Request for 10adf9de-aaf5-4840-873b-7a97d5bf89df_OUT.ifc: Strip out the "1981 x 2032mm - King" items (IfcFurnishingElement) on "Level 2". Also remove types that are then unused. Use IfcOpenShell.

First a look at what the model holds.

```python
import ifcopenshell
import ifcopenshell.util.element

model = ifcopenshell.open("10adf9de-aaf5-4840-873b-7a97d5bf89df_OUT.ifc")
print(model.schema)
storey = next(s for s in model.by_type("IfcBuildingStorey") if s.Name == "Level 2")
furniture = [e for e in ifcopenshell.util.element.get_decomposition(storey) if e.is_a("IfcFurnishingElement")]
seen = {}
for e in furniture:
    element_type = ifcopenshell.util.element.get_type(e)
    name = element_type.Name if element_type not in (None, e) else None
    seen[name] = seen.get(name, 0) + 1
for name, count in sorted(seen.items(), key=str):
    print(count, "x", name)
```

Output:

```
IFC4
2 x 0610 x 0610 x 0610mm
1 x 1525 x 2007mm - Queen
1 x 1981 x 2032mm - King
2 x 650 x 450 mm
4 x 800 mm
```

```python
import ifcopenshell
import ifcopenshell.api.root
import ifcopenshell.util.element

model = ifcopenshell.open("10adf9de-aaf5-4840-873b-7a97d5bf89df_OUT.ifc")

storey = next(s for s in model.by_type("IfcBuildingStorey") if s.Name == "Level 2")
furniture = [e for e in ifcopenshell.util.element.get_decomposition(storey) if e.is_a("IfcFurnishingElement")]
targets = [e for e in furniture if (t := ifcopenshell.util.element.get_type(e)) not in (None, e) and t.Name == "1981 x 2032mm - King"]
types = {ifcopenshell.util.element.get_type(e) for e in targets} - {None, *targets}

for e in targets:
    ifcopenshell.api.root.remove_product(model, product=e)
print(len(targets), "removed")

unused = [t for t in types if not ifcopenshell.util.element.get_types(t)]
for t in unused:
    ifcopenshell.api.root.remove_product(model, product=t)
print(len(unused), "unused types removed")

model.write("10adf9de-aaf5-4840-873b-7a97d5bf89df_OUT_updated.ifc")
```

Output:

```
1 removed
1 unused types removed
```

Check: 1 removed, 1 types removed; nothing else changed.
